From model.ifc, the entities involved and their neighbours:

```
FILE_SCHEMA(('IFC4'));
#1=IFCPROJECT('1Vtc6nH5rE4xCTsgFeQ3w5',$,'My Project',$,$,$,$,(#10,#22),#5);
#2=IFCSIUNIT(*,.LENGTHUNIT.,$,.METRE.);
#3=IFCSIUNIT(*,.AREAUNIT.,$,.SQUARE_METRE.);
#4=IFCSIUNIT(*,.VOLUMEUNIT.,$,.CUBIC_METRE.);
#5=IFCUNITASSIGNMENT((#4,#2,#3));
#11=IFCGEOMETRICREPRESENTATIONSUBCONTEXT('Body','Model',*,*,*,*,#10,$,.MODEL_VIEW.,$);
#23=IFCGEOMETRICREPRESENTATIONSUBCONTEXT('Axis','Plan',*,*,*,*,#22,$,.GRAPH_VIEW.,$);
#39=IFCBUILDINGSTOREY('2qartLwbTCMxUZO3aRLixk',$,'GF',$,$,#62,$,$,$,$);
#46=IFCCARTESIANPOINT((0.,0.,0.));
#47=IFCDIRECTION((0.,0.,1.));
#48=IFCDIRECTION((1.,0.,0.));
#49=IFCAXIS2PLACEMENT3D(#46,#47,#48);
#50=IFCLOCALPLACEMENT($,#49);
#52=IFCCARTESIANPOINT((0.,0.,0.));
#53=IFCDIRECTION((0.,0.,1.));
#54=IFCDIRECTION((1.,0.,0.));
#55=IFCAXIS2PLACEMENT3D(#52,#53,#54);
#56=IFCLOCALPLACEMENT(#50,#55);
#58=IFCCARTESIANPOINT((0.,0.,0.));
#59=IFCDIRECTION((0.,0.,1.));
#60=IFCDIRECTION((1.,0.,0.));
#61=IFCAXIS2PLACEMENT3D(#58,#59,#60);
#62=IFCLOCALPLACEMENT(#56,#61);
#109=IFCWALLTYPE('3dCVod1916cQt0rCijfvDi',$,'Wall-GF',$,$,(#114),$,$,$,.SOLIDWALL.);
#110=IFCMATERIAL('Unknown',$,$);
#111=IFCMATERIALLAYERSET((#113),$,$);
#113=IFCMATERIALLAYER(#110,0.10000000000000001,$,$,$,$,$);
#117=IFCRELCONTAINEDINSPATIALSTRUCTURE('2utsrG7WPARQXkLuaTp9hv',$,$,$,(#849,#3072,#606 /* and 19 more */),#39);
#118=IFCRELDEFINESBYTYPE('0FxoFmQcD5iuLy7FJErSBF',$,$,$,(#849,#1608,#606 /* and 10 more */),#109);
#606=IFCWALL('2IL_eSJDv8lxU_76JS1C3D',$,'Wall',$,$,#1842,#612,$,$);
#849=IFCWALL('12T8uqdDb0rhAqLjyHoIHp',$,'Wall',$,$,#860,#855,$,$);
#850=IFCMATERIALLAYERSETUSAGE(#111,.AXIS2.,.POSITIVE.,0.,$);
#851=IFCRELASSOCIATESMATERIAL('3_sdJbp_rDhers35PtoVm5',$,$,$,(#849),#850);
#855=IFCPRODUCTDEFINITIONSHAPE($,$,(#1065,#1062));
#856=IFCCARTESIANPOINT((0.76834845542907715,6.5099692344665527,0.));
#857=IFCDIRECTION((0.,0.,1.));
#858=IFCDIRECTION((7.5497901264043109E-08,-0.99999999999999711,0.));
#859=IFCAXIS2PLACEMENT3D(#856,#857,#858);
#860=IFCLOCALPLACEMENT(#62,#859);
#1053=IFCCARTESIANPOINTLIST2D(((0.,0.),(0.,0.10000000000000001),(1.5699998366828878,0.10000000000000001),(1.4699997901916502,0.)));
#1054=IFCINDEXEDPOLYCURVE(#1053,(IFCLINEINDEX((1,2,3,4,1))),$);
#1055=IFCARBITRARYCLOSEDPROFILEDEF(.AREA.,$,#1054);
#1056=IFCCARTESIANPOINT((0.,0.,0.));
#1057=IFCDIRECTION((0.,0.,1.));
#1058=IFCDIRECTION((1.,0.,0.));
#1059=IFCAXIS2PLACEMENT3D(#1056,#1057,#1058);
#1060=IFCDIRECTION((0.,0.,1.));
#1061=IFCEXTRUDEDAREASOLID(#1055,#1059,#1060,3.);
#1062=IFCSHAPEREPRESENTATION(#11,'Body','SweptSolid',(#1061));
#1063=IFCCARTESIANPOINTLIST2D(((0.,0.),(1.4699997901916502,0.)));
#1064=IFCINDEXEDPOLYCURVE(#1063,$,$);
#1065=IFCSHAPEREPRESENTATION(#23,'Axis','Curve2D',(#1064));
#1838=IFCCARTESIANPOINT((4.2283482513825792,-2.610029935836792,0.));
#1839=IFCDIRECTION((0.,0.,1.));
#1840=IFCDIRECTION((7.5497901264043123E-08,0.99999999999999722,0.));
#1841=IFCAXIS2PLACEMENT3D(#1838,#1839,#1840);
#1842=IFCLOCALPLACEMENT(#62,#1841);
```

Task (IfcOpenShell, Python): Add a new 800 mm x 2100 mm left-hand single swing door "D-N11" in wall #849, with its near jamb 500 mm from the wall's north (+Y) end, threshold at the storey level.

```python
import numpy as np
import ifcopenshell
import ifcopenshell.api.feature
import ifcopenshell.api.geometry
import ifcopenshell.api.root
import ifcopenshell.api.spatial
import ifcopenshell.geom
import ifcopenshell.util.element
import ifcopenshell.util.placement
import ifcopenshell.util.representation
import ifcopenshell.util.shape
import ifcopenshell.util.unit

model = ifcopenshell.open("model.ifc")
unit_scale = ifcopenshell.util.unit.calculate_unit_scale(model)
settings = ifcopenshell.geom.settings()


def volume(element):
    """Net volume in cubic metres, openings subtracted."""
    shape = ifcopenshell.geom.create_shape(settings, element)
    return ifcopenshell.util.shape.get_volume(shape.geometry)


wall = model.by_id(849)
storey = ifcopenshell.util.element.get_container(wall, ifc_class="IfcBuildingStorey")
context = ifcopenshell.util.representation.get_context(model, "Model", "Body", "MODEL_VIEW")
before = volume(wall)

width, height, from_end, sill = 0.8, 2.1, 0.5, 0.0  # metres

# The wall runs along its own X axis, and the end named is its -X end.
wall_shape = ifcopenshell.geom.create_shape(settings, wall)
x, y, z = ifcopenshell.util.shape.get_vertices(wall_shape.geometry).T
start = x.min() + from_end
face, thickness = float(y.min()), float(y.max() - y.min())
wall_matrix = ifcopenshell.util.placement.get_local_placement(wall.ObjectPlacement)
level = ifcopenshell.util.placement.get_local_placement(storey.ObjectPlacement)[2, 3]


def in_wall(x, y):
    """Placement at x, y metres in the wall's axes, at sill height."""
    matrix = wall_matrix.copy()
    matrix[:, 3] = wall_matrix @ np.array([x / unit_scale, y / unit_scale, 0.0, 1.0])
    matrix[2, 3] = level + sill / unit_scale
    return matrix


# Opening: a box that overshoots both wall faces by 50 mm.
opening = ifcopenshell.api.root.create_entity(model, ifc_class="IfcOpeningElement", predefined_type="OPENING")
box = ifcopenshell.api.geometry.add_wall_representation(
    model, context=context, length=width, height=height, thickness=thickness + 0.1
)
ifcopenshell.api.geometry.assign_representation(model, product=opening, representation=box)
ifcopenshell.api.geometry.edit_object_placement(model, product=opening, matrix=in_wall(start, face - 0.05), is_si=False)
ifcopenshell.api.feature.add_feature(model, feature=opening, element=wall)

door = ifcopenshell.api.root.create_entity(model, ifc_class="IfcDoor", name="D-N11", predefined_type="DOOR")
door.OverallWidth, door.OverallHeight = width / unit_scale, height / unit_scale
door.OperationType = "SINGLE_SWING_LEFT"
body = ifcopenshell.api.geometry.add_door_representation(
    model,
    context=context,
    overall_width=door.OverallWidth,
    overall_height=door.OverallHeight,
    operation_type="SINGLE_SWING_LEFT",
    lining_properties={"LiningDepth": thickness / unit_scale, "ThresholdDepth": thickness / unit_scale},
)
ifcopenshell.api.geometry.assign_representation(model, product=door, representation=body)
ifcopenshell.api.spatial.assign_container(model, products=[door], relating_structure=storey)
ifcopenshell.api.feature.add_filling(model, opening=opening, element=door)

# The lining spans the wall, so the door starts at the wall face.
ifcopenshell.api.geometry.edit_object_placement(model, product=door, matrix=in_wall(start, face), is_si=False)

after = volume(wall)

print(f"wall volume {before:.3f} -> {after:.3f} m3")

model.write("model_updated.ifc")
```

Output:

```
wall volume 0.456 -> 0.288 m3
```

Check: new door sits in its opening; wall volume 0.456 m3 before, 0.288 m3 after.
